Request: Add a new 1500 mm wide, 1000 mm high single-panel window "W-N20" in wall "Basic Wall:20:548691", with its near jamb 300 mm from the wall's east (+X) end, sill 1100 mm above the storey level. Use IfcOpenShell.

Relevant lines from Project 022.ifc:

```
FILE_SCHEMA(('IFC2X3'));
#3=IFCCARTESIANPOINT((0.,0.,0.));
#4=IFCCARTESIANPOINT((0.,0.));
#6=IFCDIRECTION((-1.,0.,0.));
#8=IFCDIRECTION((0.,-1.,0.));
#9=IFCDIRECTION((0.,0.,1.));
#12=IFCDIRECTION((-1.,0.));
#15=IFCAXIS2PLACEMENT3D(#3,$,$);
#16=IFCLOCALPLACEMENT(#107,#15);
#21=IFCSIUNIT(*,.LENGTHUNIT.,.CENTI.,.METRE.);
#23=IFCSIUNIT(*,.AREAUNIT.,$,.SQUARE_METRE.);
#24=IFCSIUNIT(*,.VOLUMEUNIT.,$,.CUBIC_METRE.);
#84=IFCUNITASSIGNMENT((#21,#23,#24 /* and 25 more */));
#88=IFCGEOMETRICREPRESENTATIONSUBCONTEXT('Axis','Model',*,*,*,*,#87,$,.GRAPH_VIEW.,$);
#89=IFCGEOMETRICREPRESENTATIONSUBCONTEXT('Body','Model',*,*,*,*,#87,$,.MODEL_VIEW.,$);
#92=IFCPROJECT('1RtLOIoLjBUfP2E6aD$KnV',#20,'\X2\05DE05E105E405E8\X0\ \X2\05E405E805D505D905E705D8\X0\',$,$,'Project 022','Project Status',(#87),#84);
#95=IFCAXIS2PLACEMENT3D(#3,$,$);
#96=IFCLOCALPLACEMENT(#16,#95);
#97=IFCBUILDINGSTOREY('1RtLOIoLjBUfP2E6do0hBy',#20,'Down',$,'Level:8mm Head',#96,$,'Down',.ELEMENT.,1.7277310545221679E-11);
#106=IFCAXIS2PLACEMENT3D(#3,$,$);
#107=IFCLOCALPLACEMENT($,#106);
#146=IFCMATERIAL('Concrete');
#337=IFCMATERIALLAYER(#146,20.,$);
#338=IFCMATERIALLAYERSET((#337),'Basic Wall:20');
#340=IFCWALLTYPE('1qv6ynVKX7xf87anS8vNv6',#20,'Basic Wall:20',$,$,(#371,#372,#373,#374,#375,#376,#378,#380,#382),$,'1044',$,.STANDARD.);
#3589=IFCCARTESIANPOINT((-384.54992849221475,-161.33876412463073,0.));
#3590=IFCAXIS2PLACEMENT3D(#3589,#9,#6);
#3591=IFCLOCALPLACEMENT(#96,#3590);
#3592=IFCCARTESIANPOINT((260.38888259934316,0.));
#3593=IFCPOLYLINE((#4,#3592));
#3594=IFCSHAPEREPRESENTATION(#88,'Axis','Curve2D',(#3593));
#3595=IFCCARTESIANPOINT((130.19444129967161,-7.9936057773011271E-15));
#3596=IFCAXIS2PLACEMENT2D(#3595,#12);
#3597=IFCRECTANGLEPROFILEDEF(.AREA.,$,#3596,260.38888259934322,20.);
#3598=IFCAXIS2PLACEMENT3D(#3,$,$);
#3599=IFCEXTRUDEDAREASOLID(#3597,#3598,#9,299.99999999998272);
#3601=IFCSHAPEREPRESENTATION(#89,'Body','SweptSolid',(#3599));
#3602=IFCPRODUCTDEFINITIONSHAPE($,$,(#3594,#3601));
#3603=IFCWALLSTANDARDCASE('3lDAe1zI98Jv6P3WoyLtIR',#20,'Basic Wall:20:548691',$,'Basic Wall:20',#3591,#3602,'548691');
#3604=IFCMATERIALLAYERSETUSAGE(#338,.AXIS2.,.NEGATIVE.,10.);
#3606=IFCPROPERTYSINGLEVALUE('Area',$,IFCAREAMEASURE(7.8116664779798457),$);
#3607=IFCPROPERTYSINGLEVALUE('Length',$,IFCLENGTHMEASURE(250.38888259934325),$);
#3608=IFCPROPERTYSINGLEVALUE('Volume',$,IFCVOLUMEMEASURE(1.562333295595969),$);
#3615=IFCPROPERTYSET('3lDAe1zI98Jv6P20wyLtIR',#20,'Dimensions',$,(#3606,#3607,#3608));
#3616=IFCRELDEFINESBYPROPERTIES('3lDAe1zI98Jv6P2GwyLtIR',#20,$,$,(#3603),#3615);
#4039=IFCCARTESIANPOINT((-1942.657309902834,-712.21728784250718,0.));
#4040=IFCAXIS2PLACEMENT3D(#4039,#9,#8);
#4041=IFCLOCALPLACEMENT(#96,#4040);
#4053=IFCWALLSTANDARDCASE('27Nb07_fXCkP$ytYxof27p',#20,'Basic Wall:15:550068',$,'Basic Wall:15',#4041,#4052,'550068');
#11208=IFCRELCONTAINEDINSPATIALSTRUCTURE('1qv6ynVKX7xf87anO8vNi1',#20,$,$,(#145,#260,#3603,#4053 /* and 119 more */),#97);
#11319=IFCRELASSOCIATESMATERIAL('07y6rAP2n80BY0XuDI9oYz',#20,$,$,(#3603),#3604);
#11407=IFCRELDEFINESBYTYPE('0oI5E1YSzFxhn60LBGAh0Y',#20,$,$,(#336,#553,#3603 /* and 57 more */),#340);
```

```python
import numpy as np
import ifcopenshell
import ifcopenshell.api.feature
import ifcopenshell.api.geometry
import ifcopenshell.api.pset
import ifcopenshell.api.root
import ifcopenshell.api.spatial
import ifcopenshell.api.type
import ifcopenshell.geom
import ifcopenshell.util.element
import ifcopenshell.util.placement
import ifcopenshell.util.representation
import ifcopenshell.util.shape
import ifcopenshell.util.unit

model = ifcopenshell.open("Project 022.ifc")
unit_scale = ifcopenshell.util.unit.calculate_unit_scale(model)
area_scale = ifcopenshell.util.unit.calculate_unit_scale(model, "AREAUNIT")
volume_scale = ifcopenshell.util.unit.calculate_unit_scale(model, "VOLUMEUNIT")
settings = ifcopenshell.geom.settings()


def volume(element):
    """Net volume in cubic metres, openings subtracted."""
    shape = ifcopenshell.geom.create_shape(settings, element)
    return ifcopenshell.util.shape.get_volume(shape.geometry)


wall = model.by_guid("3lDAe1zI98Jv6P3WoyLtIR")
storey = ifcopenshell.util.element.get_container(wall, ifc_class="IfcBuildingStorey")
context = ifcopenshell.util.representation.get_context(model, "Model", "Body", "MODEL_VIEW")
before = volume(wall)

width, height, from_end, sill = 1.5, 1, 0.3, 1.1  # metres

# The wall runs along its own X axis, and the end named is its -X end.
wall_shape = ifcopenshell.geom.create_shape(settings, wall)
x, y, z = ifcopenshell.util.shape.get_vertices(wall_shape.geometry).T
start = x.min() + from_end
face, thickness = float(y.min()), float(y.max() - y.min())
wall_matrix = ifcopenshell.util.placement.get_local_placement(wall.ObjectPlacement)
level = ifcopenshell.util.placement.get_local_placement(storey.ObjectPlacement)[2, 3]


def in_wall(x, y):
    """Placement at x, y metres in the wall's axes, at sill height."""
    matrix = wall_matrix.copy()
    matrix[:, 3] = wall_matrix @ np.array([x / unit_scale, y / unit_scale, 0.0, 1.0])
    matrix[2, 3] = level + sill / unit_scale
    return matrix


# Opening: a box that overshoots both wall faces by 50 mm.
opening = ifcopenshell.api.root.create_entity(model, ifc_class="IfcOpeningElement")
box = ifcopenshell.api.geometry.add_wall_representation(
    model, context=context, length=width, height=height, thickness=thickness + 0.1
)
ifcopenshell.api.geometry.assign_representation(model, product=opening, representation=box)
ifcopenshell.api.geometry.edit_object_placement(model, product=opening, matrix=in_wall(start, face - 0.05), is_si=False)
ifcopenshell.api.feature.add_feature(model, feature=opening, element=wall)

window = ifcopenshell.api.root.create_entity(model, ifc_class="IfcWindow", name="W-N20")
window.OverallWidth, window.OverallHeight = width / unit_scale, height / unit_scale
body = ifcopenshell.api.geometry.add_window_representation(
    model,
    context=context,
    overall_width=window.OverallWidth,
    overall_height=window.OverallHeight,
    partition_type="SINGLE_PANEL",
)
ifcopenshell.api.geometry.assign_representation(model, product=window, representation=body)
ifcopenshell.api.spatial.assign_container(model, products=[window], relating_structure=storey)
fills = ifcopenshell.api.feature.add_filling(model, opening=opening, element=window)
fills.OwnerHistory = window.OwnerHistory  # required in IFC2X3

# IFC2X3 keeps the operation on the window style.
style = ifcopenshell.api.root.create_entity(model, ifc_class="IfcWindowStyle", name="W-N20")
style.OperationType, style.ConstructionType = "SINGLE_PANEL", "NOTDEFINED"
style.ParameterTakesPrecedence = style.Sizeable = False
ifcopenshell.api.type.assign_type(model, related_objects=[window], relating_type=style)

# Centre the window in the wall's thickness.
ifcopenshell.api.geometry.edit_object_placement(model, product=window, matrix=in_wall(start, face), is_si=False)
window_shape = ifcopenshell.geom.create_shape(settings, window)
depth = ifcopenshell.util.shape.get_vertices(window_shape.geometry)[:, 1]
offset = face + thickness / 2 - (depth.min() + depth.max()) / 2
ifcopenshell.api.geometry.edit_object_placement(model, product=window, matrix=in_wall(start, offset), is_si=False)

after = volume(wall)

# Update the wall's stored quantities.
pset = model.by_id(ifcopenshell.util.element.get_pset(wall, "Dimensions", should_inherit=False)["id"])
ifcopenshell.api.pset.edit_pset(model, pset=pset, properties={
    "Area": model.create_entity("IfcAreaMeasure", after / thickness / area_scale),
    "Volume": model.create_entity("IfcVolumeMeasure", after / volume_scale),
})

print(f"wall volume {before:.3f} -> {after:.3f} m3")

model.write("Project 022-out.ifc")
```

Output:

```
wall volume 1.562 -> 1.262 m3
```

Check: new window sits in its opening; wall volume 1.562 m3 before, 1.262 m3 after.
